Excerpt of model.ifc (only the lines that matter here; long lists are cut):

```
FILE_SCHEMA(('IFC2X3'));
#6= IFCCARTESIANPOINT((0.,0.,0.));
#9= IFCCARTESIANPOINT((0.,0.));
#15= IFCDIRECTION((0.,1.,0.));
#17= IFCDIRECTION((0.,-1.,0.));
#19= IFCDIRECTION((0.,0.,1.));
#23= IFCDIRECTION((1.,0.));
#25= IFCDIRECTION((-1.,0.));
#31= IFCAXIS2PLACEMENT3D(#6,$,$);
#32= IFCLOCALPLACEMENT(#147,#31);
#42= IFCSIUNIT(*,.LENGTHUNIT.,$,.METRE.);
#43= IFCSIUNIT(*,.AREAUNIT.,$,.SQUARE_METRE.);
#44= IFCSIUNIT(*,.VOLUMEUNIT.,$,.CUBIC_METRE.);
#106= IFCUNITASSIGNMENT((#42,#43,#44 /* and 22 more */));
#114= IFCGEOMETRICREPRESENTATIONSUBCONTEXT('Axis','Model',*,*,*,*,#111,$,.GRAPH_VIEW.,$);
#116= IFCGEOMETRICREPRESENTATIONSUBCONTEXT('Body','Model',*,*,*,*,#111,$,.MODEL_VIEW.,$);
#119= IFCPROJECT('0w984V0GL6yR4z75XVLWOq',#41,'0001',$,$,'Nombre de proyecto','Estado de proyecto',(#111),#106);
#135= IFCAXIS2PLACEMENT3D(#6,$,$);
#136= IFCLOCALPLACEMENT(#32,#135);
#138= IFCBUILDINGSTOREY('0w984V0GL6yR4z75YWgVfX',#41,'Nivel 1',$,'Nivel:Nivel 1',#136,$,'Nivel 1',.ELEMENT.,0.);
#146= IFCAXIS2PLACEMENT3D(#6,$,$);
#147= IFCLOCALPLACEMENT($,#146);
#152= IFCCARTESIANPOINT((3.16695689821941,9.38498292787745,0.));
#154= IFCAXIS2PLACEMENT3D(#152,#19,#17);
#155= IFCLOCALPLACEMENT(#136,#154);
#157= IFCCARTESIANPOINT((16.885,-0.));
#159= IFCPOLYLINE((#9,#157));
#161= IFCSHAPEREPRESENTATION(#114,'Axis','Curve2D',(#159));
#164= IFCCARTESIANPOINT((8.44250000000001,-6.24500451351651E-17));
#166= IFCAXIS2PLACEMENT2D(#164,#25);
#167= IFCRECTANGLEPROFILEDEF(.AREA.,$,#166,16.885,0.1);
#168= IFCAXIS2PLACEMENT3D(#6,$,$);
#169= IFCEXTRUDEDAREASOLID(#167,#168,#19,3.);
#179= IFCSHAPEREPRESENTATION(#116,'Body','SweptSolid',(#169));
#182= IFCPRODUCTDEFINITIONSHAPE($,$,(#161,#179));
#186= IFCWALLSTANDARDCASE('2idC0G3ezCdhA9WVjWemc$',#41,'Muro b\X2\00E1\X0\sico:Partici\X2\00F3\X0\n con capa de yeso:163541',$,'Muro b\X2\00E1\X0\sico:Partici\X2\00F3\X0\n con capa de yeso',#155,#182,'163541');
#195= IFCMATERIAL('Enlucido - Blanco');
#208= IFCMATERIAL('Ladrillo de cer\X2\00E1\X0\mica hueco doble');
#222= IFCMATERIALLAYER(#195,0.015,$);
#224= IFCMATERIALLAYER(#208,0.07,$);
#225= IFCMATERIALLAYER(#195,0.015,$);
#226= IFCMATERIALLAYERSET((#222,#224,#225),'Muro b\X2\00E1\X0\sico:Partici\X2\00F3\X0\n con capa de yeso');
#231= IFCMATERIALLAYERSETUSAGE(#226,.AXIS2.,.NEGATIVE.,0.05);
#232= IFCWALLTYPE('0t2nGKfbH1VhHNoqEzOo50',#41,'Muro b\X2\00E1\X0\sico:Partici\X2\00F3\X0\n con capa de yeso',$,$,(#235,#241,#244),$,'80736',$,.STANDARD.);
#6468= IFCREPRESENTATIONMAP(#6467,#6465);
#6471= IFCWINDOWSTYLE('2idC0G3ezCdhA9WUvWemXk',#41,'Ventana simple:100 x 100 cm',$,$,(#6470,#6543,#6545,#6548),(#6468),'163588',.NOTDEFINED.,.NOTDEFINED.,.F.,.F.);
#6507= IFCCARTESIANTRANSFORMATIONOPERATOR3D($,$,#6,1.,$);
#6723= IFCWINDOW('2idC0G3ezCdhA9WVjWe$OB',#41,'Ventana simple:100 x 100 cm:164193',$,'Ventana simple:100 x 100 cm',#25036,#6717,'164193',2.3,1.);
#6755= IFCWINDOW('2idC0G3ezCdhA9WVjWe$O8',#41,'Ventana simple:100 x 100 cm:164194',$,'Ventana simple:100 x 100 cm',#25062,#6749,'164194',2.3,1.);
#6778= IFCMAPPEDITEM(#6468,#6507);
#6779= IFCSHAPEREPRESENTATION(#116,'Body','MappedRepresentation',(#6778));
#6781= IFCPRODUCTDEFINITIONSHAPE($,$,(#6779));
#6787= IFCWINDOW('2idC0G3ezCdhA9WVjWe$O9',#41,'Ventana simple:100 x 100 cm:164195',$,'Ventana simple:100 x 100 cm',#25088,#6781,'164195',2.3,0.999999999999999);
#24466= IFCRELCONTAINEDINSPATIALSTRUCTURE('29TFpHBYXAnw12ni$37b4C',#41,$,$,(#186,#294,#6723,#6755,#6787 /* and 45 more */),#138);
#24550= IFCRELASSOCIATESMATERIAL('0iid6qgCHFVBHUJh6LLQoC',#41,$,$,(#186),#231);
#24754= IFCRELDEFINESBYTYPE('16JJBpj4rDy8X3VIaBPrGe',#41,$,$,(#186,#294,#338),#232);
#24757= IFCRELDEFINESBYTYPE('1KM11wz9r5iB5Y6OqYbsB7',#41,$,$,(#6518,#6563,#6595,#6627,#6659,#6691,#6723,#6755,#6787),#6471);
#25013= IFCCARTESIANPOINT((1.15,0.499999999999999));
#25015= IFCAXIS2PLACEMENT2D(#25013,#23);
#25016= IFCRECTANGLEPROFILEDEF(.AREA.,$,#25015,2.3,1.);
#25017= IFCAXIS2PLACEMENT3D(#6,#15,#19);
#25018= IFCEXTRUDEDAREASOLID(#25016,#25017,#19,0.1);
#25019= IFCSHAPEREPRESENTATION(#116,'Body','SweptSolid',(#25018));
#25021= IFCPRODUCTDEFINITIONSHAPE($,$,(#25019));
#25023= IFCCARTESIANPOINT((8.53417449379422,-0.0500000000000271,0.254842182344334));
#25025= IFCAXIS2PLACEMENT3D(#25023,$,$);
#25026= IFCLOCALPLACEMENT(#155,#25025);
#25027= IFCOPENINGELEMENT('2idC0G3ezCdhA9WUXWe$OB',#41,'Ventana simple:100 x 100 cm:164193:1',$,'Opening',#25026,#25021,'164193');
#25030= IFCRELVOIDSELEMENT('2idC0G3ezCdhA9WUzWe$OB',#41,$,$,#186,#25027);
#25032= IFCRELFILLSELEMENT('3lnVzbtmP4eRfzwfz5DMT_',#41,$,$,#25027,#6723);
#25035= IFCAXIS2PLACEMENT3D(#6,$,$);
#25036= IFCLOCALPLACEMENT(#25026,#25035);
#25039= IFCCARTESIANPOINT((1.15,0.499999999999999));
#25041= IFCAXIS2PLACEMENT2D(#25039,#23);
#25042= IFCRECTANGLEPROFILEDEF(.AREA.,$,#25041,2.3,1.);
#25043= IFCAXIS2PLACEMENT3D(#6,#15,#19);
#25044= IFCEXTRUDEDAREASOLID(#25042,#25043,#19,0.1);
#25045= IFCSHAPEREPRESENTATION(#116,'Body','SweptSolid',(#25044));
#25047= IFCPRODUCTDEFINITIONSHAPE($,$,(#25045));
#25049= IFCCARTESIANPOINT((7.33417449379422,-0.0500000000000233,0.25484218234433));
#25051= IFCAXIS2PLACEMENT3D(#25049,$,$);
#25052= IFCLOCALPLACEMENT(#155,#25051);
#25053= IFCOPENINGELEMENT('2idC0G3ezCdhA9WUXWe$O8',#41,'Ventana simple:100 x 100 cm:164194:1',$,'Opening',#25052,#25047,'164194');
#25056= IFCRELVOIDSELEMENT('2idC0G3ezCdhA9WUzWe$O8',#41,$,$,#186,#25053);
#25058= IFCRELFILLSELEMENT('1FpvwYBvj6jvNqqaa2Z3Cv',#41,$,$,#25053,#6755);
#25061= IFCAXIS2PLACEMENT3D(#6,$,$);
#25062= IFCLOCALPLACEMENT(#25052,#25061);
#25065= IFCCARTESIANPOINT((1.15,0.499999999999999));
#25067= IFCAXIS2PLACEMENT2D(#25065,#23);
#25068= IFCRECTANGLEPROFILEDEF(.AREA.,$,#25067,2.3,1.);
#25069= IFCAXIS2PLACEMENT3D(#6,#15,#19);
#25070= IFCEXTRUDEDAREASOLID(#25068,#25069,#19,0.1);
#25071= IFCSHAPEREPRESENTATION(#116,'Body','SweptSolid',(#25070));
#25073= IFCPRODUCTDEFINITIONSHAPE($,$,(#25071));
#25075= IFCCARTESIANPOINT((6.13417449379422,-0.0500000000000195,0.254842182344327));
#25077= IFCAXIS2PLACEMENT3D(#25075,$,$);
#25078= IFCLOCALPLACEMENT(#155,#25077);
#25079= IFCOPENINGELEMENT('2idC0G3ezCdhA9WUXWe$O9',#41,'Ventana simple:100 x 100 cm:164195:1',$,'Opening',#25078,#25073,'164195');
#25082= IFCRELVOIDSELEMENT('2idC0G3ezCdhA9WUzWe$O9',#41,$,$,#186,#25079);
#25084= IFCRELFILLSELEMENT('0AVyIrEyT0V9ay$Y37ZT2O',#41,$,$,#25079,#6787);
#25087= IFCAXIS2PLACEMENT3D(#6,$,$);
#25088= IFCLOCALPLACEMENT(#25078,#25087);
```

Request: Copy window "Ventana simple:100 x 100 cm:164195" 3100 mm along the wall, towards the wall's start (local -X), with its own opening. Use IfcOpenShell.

```python
import ifcopenshell
import ifcopenshell.api.feature
import ifcopenshell.api.geometry
import ifcopenshell.api.root
import ifcopenshell.geom
import ifcopenshell.util.element
import ifcopenshell.util.placement
import ifcopenshell.util.shape

model = ifcopenshell.open("model.ifc")
settings = ifcopenshell.geom.settings()


def volume(element):
    """Net volume in cubic metres, openings subtracted."""
    shape = ifcopenshell.geom.create_shape(settings, element)
    return ifcopenshell.util.shape.get_volume(shape.geometry)


def reuse_history(source, copy):
    """copy_class also copies each property set's owner history, people and application; keep the originals."""
    for rel in copy.IsDefinedBy:
        if rel.is_a("IfcRelDefinesByProperties") and (history := rel.RelatingPropertyDefinition.OwnerHistory):
            rel.RelatingPropertyDefinition.OwnerHistory = source.OwnerHistory
            ifcopenshell.util.element.remove_deep2(model, history)


window = model.by_guid("2idC0G3ezCdhA9WVjWe$O9")
opening = window.FillsVoids[0].RelatingOpeningElement
wall = opening.VoidsElements[0].RelatingBuildingElement
before = volume(wall)
shift = ifcopenshell.util.placement.get_local_placement(wall.ObjectPlacement)[:3, 0] * -3.1

# copy_class copies the void relationship, type, container and properties, but no geometry.
new_opening = ifcopenshell.api.root.copy_class(model, product=opening)
new_opening.Representation = ifcopenshell.util.element.copy_deep(
    model, opening.Representation, exclude=["IfcGeometricRepresentationContext", "IfcRepresentationMap"]
)
new_opening.Name = "Ventana simple:100 x 100 cm"
new_opening.Tag = None
new_window = ifcopenshell.api.root.copy_class(model, product=window)
new_window.Representation = ifcopenshell.util.element.copy_deep(
    model, window.Representation, exclude=["IfcGeometricRepresentationContext", "IfcRepresentationMap"]
)
new_window.Name = "Ventana simple:100 x 100 cm"
new_window.Tag = None
reuse_history(window, new_window)
fills = ifcopenshell.api.feature.add_filling(model, opening=new_opening, element=new_window)
fills.OwnerHistory = new_window.OwnerHistory  # required in IFC2X3

for old, new in ((opening, new_opening), (window, new_window)):
    matrix = ifcopenshell.util.placement.get_local_placement(old.ObjectPlacement)
    matrix[:3, 3] += shift
    ifcopenshell.api.geometry.edit_object_placement(model, product=new, matrix=matrix, is_si=False)

after = volume(wall)

print(f"wall volume {before:.3f} -> {after:.3f} m3")

model.write("model-out.ifc")
```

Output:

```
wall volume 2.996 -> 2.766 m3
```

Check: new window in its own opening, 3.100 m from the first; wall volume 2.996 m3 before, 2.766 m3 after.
